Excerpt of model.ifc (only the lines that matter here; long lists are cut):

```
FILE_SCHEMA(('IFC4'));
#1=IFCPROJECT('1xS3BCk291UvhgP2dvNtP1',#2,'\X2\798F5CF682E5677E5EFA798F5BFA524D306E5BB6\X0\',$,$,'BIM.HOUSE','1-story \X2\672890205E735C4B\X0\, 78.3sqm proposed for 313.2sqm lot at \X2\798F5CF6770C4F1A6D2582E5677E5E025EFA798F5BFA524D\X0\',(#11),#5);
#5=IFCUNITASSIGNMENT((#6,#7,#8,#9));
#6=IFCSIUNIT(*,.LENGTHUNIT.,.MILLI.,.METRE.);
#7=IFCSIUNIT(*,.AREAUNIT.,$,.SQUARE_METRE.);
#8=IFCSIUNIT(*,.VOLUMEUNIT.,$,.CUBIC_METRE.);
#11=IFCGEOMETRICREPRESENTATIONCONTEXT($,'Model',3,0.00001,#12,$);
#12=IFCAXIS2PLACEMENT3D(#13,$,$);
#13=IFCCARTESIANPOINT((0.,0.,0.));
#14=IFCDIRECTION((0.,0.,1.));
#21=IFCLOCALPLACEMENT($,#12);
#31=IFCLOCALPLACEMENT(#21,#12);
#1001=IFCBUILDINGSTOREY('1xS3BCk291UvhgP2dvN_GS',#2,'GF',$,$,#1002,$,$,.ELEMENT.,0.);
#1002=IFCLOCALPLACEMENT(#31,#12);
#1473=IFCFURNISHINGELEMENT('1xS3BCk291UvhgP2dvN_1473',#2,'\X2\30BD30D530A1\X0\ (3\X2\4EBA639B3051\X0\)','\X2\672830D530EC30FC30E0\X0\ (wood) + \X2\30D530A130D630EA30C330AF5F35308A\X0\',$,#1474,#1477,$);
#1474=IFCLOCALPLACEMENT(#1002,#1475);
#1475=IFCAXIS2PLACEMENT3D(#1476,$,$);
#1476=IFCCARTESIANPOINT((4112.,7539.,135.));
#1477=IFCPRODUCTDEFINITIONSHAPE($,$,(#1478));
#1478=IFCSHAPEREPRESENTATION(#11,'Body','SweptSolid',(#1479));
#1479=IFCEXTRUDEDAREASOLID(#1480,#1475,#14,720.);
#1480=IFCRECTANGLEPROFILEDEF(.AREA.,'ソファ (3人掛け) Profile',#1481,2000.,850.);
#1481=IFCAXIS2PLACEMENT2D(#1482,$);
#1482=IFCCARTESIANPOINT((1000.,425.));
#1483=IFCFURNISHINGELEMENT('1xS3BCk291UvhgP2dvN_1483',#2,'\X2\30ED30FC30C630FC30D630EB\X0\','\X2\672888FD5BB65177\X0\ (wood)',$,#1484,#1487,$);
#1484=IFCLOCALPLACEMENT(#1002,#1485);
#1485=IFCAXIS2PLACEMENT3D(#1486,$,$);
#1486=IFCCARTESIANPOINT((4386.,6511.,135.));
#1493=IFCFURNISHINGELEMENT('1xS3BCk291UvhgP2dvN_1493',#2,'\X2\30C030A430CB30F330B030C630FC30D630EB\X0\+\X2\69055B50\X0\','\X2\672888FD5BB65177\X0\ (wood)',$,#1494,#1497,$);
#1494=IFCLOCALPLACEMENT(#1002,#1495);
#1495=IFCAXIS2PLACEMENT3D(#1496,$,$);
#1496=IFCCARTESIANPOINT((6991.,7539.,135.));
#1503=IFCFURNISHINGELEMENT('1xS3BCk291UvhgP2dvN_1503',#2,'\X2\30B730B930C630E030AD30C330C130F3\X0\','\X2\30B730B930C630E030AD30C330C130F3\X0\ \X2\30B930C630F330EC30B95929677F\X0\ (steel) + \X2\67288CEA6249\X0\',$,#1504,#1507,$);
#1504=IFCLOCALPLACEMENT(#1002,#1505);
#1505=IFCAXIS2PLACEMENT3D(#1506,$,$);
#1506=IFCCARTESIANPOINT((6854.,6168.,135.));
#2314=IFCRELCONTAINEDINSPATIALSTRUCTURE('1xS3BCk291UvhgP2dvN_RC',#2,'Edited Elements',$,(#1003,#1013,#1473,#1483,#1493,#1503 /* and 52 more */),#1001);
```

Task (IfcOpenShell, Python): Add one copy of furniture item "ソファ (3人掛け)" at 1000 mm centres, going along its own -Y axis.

```python
import ifcopenshell
import ifcopenshell.api.geometry
import ifcopenshell.api.root
import ifcopenshell.util.element
import ifcopenshell.util.placement

model = ifcopenshell.open("model.ifc")


def reuse_history(source, copy):
    """copy_class also copies each property set's owner history, people and application; keep the originals."""
    for rel in copy.IsDefinedBy:
        if rel.is_a("IfcRelDefinesByProperties") and (history := rel.RelatingPropertyDefinition.OwnerHistory):
            rel.RelatingPropertyDefinition.OwnerHistory = source.OwnerHistory
            ifcopenshell.util.element.remove_deep2(model, history)


source = model.by_guid("1xS3BCk291UvhgP2dvN_1473")
base = ifcopenshell.util.placement.get_local_placement(source.ObjectPlacement)
step = -base[:3, 1] * 1000.0

for i in range(1, 2):
    copy = ifcopenshell.api.root.copy_class(model, product=source)
    copy.Representation = ifcopenshell.util.element.copy_deep(
        model, source.Representation, exclude=["IfcGeometricRepresentationContext", "IfcRepresentationMap"]
    )
    reuse_history(source, copy)
    matrix = base.copy()
    matrix[:3, 3] += i * step
    print("added at", matrix[:3, 3].round(3) + 0.0)
    ifcopenshell.api.geometry.edit_object_placement(model, product=copy, matrix=matrix, is_si=False)

model.write("model_updated.ifc")
```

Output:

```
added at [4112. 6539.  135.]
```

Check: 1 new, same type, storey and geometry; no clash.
